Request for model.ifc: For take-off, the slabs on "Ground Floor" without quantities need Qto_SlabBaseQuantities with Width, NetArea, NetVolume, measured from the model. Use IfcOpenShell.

First a look at what the model holds.

```python
import ifcopenshell
import ifcopenshell.util.element
import ifcopenshell.util.unit

model = ifcopenshell.open("model.ifc")
print(model.schema)
for unit_type in ("LENGTHUNIT", "AREAUNIT", "VOLUMEUNIT"):
    print(unit_type, ifcopenshell.util.unit.calculate_unit_scale(model, unit_type))
storey = next(s for s in model.by_type("IfcBuildingStorey") if s.Name == "Ground Floor")
slabs = [e for e in ifcopenshell.util.element.get_decomposition(storey) if e.is_a("IfcSlab")]
for e in sorted(slabs, key=lambda e: e.id()):
    print(e.id(), e.is_a(), e.Name, list(ifcopenshell.util.element.get_psets(e, qtos_only=True)), sep=" | ")
```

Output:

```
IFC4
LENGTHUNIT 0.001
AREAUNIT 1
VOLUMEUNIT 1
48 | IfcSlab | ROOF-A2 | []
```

```python
import ifcopenshell
import ifcopenshell.api.pset
import ifcopenshell.geom
import ifcopenshell.util.element
import ifcopenshell.util.shape
import ifcopenshell.util.unit

model = ifcopenshell.open("model.ifc")
unit_scale = ifcopenshell.util.unit.calculate_unit_scale(model)
area_scale = ifcopenshell.util.unit.calculate_unit_scale(model, "AREAUNIT")
volume_scale = ifcopenshell.util.unit.calculate_unit_scale(model, "VOLUMEUNIT")
settings = ifcopenshell.geom.settings()

storey = next(s for s in model.by_type("IfcBuildingStorey") if s.Name == "Ground Floor")
slabs = [e for e in ifcopenshell.util.element.get_decomposition(storey) if e.is_a("IfcSlab")]

for e in sorted(slabs, key=lambda e: e.id()):
    if ifcopenshell.util.element.get_psets(e, qtos_only=True, should_inherit=False):
        continue
    # Geometry comes back in metres, in the element's own axes.
    shape = ifcopenshell.geom.create_shape(settings, e)
    values = {
        "Width": ifcopenshell.util.shape.get_z(shape.geometry) / unit_scale,
        "NetArea": ifcopenshell.util.shape.get_footprint_area(shape.geometry) / area_scale,
        "NetVolume": ifcopenshell.util.shape.get_volume(shape.geometry) / volume_scale,
    }
    qto = ifcopenshell.api.pset.add_qto(model, product=e, name="Qto_SlabBaseQuantities")
    ifcopenshell.api.pset.edit_qto(model, qto=qto, properties=values)
    print(e.id(), {k: round(v, 3) for k, v in values.items()})

model.write("model_updated.ifc")
```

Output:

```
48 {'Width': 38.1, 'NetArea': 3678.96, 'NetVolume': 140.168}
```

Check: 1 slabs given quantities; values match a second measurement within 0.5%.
